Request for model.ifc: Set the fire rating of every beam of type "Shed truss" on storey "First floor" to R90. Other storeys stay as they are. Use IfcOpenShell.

First a look at what the model holds.

```python
import ifcopenshell
import ifcopenshell.util.element

model = ifcopenshell.open("model.ifc")
print(model.schema)
storey = next(s for s in model.by_type("IfcBuildingStorey") if s.Name == "First floor")
beams = [e for e in ifcopenshell.util.element.get_decomposition(storey) if e.is_a("IfcBeam")]
seen = {}
for e in beams:
    element_type = ifcopenshell.util.element.get_type(e)
    key = (element_type.Name if element_type != e and element_type else None, ifcopenshell.util.element.get_pset(e, "Pset_BeamCommon", "FireRating"))
    seen[key] = seen.get(key, 0) + 1
for (name, value), count in sorted(seen.items(), key=str):
    print(count, "x", name, "|", value)
```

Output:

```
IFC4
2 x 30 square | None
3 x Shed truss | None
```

```python
import ifcopenshell
import ifcopenshell.api.pset
import ifcopenshell.util.element

model = ifcopenshell.open("model.ifc")

storey = next(s for s in model.by_type("IfcBuildingStorey") if s.Name == "First floor")
beams = [e for e in ifcopenshell.util.element.get_decomposition(storey) if e.is_a("IfcBeam")]

count = 0
for e in beams:
    element_type = ifcopenshell.util.element.get_type(e)
    if element_type in (None, e) or element_type.Name != "Shed truss":
        continue
    # add_pset returns the element's existing set when there is one.
    pset = ifcopenshell.api.pset.add_pset(model, product=e, name="Pset_BeamCommon")
    ifcopenshell.api.pset.edit_pset(model, pset=pset, properties={"FireRating": "R90"})
    count += 1

print(count, "beams updated")

model.write("model_edited.ifc")
```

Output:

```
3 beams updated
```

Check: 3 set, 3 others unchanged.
